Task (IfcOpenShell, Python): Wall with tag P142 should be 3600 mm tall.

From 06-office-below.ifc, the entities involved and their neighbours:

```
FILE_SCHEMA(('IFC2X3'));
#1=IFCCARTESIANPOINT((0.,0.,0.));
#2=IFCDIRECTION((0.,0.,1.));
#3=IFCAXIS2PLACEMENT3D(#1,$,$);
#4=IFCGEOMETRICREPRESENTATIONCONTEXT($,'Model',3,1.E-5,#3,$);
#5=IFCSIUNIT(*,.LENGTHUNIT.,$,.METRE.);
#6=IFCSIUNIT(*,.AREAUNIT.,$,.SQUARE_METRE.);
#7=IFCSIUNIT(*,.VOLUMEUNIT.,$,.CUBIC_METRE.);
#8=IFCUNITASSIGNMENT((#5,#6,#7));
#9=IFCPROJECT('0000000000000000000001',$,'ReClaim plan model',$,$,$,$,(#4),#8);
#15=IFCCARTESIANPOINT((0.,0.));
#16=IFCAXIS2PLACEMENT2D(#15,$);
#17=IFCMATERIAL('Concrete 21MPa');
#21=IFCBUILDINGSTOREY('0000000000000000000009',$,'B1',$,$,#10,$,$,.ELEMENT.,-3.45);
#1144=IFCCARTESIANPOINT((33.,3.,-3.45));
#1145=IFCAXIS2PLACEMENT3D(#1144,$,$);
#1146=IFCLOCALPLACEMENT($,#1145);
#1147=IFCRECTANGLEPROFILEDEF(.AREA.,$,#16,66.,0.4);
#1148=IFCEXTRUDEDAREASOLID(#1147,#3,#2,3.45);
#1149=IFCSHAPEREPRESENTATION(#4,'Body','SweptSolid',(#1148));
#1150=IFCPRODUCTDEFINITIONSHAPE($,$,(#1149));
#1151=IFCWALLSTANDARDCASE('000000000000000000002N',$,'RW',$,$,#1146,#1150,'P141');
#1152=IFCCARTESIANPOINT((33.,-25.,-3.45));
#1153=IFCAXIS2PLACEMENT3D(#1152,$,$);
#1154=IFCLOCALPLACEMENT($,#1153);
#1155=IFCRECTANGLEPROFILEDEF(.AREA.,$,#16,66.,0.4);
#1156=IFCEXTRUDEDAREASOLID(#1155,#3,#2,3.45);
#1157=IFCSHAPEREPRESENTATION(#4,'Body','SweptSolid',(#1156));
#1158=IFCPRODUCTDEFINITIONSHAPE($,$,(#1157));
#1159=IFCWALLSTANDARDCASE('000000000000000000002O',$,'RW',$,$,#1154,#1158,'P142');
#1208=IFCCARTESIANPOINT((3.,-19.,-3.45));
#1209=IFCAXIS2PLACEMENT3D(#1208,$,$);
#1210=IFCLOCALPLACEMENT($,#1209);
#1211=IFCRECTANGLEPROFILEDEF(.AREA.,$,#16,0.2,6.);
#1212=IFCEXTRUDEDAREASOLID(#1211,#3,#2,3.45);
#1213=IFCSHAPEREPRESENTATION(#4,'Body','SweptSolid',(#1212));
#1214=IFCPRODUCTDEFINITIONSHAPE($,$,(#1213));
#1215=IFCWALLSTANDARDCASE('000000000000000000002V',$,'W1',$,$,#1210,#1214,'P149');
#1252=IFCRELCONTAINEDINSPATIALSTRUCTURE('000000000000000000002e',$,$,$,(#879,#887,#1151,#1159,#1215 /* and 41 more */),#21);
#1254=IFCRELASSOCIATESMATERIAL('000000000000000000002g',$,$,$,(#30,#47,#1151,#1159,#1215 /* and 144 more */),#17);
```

```python
import ifcopenshell
import ifcopenshell.geom
import ifcopenshell.util.shape
import ifcopenshell.util.unit

model = ifcopenshell.open("06-office-below.ifc")
unit_scale = ifcopenshell.util.unit.calculate_unit_scale(model)
settings = ifcopenshell.geom.settings()


def volume(element):
    """Net volume in cubic metres, openings subtracted."""
    shape = ifcopenshell.geom.create_shape(settings, element)
    return ifcopenshell.util.shape.get_volume(shape.geometry)


wall = model.by_id(1159)
before = volume(wall)

body = next(r for r in wall.Representation.Representations if r.RepresentationIdentifier == "Body")
solid = body.Items[0]
old_height = solid.Depth
solid.Depth = 3.6 / unit_scale
after = volume(wall)

print(f"height {old_height:g} -> {solid.Depth:g}, volume {before:.3f} -> {after:.3f} m3")

model.write("06-office-below_updated.ifc")
```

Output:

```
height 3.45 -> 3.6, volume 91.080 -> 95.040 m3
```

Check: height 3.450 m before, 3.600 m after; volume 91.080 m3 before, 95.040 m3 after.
